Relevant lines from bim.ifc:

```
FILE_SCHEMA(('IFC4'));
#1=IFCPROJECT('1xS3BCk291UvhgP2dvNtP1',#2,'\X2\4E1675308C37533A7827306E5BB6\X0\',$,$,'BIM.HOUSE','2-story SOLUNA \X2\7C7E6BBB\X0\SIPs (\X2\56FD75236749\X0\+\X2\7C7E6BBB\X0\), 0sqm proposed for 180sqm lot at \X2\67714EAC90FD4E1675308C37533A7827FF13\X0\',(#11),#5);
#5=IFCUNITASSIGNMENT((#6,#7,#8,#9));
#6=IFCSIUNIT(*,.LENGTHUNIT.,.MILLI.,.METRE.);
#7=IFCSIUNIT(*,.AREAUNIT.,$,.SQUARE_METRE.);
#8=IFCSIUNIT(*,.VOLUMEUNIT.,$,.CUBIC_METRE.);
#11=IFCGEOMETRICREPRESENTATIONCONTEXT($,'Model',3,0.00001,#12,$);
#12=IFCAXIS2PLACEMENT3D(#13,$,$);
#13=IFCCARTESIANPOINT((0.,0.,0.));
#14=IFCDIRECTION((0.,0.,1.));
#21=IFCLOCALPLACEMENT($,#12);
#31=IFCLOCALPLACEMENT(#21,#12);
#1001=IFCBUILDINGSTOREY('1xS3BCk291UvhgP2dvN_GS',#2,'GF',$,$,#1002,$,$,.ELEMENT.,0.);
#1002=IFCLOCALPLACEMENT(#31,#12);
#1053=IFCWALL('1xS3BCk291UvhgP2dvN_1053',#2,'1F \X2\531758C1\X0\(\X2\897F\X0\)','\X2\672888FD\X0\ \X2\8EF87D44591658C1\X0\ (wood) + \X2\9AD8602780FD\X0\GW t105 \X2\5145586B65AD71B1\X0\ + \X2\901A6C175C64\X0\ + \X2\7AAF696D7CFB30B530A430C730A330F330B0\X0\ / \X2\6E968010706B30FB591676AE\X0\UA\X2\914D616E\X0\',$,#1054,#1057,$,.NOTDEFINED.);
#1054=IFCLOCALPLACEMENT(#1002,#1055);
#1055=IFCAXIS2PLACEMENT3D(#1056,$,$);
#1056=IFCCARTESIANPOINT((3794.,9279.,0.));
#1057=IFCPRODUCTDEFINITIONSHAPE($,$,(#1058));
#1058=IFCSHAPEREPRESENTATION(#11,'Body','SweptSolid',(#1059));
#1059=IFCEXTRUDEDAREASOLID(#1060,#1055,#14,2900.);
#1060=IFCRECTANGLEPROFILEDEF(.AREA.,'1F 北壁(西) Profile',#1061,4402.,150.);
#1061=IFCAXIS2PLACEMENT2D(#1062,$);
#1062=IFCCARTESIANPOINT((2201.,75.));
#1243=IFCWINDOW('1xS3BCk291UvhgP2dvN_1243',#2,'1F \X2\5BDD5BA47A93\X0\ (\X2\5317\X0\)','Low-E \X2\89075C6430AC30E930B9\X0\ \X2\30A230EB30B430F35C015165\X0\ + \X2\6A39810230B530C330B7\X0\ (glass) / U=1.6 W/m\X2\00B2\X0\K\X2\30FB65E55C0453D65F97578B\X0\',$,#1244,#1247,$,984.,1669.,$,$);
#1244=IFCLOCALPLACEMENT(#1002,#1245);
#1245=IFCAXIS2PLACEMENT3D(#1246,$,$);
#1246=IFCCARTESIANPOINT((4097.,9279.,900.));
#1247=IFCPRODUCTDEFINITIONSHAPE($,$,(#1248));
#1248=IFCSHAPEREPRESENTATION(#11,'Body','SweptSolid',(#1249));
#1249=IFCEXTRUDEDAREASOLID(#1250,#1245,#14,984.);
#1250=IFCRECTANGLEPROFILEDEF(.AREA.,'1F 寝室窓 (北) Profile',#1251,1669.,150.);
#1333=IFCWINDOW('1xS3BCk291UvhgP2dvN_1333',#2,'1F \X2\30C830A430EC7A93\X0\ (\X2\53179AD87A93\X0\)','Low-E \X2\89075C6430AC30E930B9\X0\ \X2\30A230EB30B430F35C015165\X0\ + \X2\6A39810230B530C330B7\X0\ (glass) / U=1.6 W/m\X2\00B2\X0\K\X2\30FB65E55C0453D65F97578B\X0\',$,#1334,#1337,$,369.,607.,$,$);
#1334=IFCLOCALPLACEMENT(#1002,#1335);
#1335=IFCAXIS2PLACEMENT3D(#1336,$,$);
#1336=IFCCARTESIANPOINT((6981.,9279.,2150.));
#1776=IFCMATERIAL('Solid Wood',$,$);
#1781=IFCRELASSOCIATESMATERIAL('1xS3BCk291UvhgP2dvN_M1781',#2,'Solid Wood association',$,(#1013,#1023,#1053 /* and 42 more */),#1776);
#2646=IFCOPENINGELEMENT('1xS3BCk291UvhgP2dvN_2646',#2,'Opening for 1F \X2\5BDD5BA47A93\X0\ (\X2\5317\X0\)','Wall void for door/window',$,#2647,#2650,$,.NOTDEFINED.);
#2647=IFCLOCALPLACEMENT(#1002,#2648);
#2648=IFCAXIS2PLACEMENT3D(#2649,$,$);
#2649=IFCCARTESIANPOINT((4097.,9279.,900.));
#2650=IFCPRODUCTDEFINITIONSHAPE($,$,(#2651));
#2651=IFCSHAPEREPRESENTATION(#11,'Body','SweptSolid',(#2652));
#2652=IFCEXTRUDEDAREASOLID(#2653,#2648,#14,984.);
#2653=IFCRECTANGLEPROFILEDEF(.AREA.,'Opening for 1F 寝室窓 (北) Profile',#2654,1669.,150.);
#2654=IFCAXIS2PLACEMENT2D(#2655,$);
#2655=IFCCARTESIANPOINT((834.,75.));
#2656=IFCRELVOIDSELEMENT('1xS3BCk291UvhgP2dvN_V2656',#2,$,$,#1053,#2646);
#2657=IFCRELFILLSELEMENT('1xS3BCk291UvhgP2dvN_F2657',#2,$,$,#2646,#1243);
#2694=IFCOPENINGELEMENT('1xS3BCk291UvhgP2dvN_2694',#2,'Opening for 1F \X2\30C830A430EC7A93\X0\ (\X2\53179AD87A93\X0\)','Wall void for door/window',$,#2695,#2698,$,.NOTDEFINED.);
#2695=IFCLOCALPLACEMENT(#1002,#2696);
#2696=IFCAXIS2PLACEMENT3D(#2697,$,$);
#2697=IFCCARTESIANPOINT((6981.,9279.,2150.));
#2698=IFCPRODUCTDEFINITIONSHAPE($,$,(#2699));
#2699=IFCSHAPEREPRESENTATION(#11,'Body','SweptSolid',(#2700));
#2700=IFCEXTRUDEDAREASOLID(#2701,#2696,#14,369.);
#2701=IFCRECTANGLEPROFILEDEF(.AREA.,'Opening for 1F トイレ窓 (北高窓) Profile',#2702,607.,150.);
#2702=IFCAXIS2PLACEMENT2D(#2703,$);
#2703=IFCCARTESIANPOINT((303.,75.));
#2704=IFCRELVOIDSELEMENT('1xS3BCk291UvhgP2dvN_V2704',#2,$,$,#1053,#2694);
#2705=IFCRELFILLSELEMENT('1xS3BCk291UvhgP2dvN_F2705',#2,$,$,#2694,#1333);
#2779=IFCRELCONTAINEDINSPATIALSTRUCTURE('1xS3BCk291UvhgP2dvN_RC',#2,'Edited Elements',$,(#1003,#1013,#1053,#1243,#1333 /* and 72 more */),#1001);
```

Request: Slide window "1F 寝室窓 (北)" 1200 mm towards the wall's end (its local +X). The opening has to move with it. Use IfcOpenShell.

```python
import ifcopenshell
import ifcopenshell.api.geometry
import ifcopenshell.util.placement

model = ifcopenshell.open("bim.ifc")

window = model.by_guid("1xS3BCk291UvhgP2dvN_1243")
opening = window.FillsVoids[0].RelatingOpeningElement
wall = opening.VoidsElements[0].RelatingBuildingElement

wall_matrix = ifcopenshell.util.placement.get_local_placement(wall.ObjectPlacement)
shift = wall_matrix[:3, 0] * 1200.0
before = ifcopenshell.util.placement.get_local_placement(window.ObjectPlacement)[:3, 3].copy()

# The window is not placed relative to its opening, so move both.
for product in (opening, window):
    matrix = ifcopenshell.util.placement.get_local_placement(product.ObjectPlacement)
    matrix[:3, 3] += shift
    ifcopenshell.api.geometry.edit_object_placement(model, product=product, matrix=matrix, is_si=False)

after = ifcopenshell.util.placement.get_local_placement(window.ObjectPlacement)[:3, 3]
print("window moved by", (after - before).round(3) + 0.0)

model.write("bim_rev.ifc")
```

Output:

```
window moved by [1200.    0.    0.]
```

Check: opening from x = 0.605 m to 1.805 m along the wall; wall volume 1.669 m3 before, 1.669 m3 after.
